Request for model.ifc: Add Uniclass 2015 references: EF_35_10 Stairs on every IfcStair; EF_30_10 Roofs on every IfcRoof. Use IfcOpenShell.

First a look at what the model holds.

```python
import ifcopenshell

model = ifcopenshell.open("model.ifc")
print(model.schema)
print("classifications:", [c.Name for c in model.by_type("IfcClassification")])
for ifc_class in ("IfcDoor", "IfcRoof", "IfcStair", "IfcWall", "IfcWindow"):
    print(ifc_class, len(model.by_type(ifc_class)))
```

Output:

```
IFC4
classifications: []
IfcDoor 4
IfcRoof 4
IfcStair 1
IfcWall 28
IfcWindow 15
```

```python
import ifcopenshell
import ifcopenshell.api.classification

model = ifcopenshell.open("model.ifc")

system = ifcopenshell.api.classification.add_classification(model, classification="Uniclass 2015")

codes = {
    "IfcStair": ("EF_35_10", "Stairs"),
    "IfcRoof": ("EF_30_10", "Roofs"),
}
for ifc_class, (code, name) in codes.items():
    products = model.by_type(ifc_class)
    ifcopenshell.api.classification.add_reference(
        model, products=products, classification=system, identification=code, name=name
    )
    print(code, len(products))

model.write("model_rev.ifc")
```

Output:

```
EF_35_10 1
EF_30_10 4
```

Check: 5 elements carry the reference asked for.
